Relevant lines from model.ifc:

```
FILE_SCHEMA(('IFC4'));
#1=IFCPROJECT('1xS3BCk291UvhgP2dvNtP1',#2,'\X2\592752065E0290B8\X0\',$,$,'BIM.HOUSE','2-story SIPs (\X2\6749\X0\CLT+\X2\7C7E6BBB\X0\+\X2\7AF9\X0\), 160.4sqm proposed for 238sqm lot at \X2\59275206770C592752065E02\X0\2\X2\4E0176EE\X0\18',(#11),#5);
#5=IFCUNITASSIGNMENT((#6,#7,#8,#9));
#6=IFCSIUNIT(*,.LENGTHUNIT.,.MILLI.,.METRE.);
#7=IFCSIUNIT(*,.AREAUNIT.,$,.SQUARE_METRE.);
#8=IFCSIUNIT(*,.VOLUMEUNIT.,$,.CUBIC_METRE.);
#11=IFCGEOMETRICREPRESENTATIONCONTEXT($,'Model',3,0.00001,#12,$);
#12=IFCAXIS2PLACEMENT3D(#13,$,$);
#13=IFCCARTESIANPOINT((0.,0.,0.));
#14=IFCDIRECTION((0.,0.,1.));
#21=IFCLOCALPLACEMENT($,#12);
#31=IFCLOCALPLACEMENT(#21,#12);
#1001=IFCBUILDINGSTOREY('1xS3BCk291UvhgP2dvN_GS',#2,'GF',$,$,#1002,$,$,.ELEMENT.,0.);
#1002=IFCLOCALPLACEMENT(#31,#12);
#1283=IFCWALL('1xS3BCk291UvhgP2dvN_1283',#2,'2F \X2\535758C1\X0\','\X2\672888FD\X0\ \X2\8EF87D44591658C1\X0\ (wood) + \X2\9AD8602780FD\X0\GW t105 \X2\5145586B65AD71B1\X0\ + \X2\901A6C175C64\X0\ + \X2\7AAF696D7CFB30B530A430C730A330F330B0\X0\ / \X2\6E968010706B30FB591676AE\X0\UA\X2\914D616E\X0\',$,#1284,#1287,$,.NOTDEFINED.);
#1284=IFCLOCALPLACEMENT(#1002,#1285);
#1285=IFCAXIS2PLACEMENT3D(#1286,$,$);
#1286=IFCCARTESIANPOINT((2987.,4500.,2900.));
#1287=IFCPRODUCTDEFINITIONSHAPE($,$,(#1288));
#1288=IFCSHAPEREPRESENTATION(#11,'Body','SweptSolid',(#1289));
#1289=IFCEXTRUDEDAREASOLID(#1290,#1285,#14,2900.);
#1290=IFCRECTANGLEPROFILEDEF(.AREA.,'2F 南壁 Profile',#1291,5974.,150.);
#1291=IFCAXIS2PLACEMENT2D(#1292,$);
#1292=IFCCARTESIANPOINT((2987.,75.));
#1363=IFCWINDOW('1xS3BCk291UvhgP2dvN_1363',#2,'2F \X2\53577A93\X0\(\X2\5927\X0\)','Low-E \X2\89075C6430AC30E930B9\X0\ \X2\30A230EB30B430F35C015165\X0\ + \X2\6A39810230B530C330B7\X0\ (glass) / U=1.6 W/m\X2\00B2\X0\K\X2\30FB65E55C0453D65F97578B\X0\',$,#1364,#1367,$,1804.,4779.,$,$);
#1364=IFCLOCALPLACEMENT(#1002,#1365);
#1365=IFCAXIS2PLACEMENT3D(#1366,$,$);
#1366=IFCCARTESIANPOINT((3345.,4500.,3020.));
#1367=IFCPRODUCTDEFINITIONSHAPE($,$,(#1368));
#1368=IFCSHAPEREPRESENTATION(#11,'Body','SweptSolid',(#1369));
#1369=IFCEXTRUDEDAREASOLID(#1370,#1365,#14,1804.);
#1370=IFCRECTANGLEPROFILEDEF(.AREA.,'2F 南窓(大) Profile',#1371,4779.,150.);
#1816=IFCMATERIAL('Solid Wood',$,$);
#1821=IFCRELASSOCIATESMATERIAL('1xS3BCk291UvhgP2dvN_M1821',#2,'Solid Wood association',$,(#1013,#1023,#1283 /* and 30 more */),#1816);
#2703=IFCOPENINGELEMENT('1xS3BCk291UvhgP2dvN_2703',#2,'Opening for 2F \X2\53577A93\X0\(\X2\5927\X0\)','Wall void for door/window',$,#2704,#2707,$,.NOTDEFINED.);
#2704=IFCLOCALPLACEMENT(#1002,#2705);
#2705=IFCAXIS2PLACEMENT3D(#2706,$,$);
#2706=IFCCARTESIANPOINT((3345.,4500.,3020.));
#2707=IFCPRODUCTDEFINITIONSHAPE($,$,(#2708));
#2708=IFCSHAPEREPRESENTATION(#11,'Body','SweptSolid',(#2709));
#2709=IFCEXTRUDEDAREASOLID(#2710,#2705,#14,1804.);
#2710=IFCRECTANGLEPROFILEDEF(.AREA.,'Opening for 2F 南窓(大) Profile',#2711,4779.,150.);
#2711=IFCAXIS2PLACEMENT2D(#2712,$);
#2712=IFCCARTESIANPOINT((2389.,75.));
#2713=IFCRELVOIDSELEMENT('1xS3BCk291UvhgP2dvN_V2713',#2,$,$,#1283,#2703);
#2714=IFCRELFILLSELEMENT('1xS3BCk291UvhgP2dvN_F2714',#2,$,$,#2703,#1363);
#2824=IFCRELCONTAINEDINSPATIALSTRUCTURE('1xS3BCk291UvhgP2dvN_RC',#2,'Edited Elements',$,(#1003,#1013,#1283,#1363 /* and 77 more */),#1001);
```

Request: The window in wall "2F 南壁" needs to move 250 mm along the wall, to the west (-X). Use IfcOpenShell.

```python
import ifcopenshell
import ifcopenshell.api.geometry
import ifcopenshell.util.placement
import ifcopenshell.util.unit

model = ifcopenshell.open("model.ifc")
unit_scale = ifcopenshell.util.unit.calculate_unit_scale(model)

window = model.by_guid("1xS3BCk291UvhgP2dvN_1363")
opening = window.FillsVoids[0].RelatingOpeningElement
wall = opening.VoidsElements[0].RelatingBuildingElement

wall_matrix = ifcopenshell.util.placement.get_local_placement(wall.ObjectPlacement)
shift = wall_matrix[:3, 0] * -0.25 / unit_scale
before = ifcopenshell.util.placement.get_local_placement(window.ObjectPlacement)[:3, 3].copy()

# The window is not placed relative to its opening, so move both.
for product in (opening, window):
    matrix = ifcopenshell.util.placement.get_local_placement(product.ObjectPlacement)
    matrix[:3, 3] += shift
    ifcopenshell.api.geometry.edit_object_placement(model, product=product, matrix=matrix, is_si=False)

after = ifcopenshell.util.placement.get_local_placement(window.ObjectPlacement)[:3, 3]
print("window moved by", (after - before).round(3) + 0.0)

model.write("model_v2.ifc")
```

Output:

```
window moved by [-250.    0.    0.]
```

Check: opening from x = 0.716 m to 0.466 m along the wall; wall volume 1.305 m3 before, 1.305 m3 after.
